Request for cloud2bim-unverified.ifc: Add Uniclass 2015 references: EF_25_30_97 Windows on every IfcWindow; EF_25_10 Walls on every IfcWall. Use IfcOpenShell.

First a look at what the model holds.

```python
import ifcopenshell

model = ifcopenshell.open("cloud2bim-unverified.ifc")
print(model.schema)
print("classifications:", [c.Name for c in model.by_type("IfcClassification")])
for ifc_class in ("IfcDoor", "IfcRoof", "IfcStair", "IfcWall", "IfcWindow"):
    print(ifc_class, len(model.by_type(ifc_class)))
```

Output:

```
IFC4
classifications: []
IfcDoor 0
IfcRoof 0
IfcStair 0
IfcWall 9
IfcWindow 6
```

```python
import ifcopenshell
import ifcopenshell.api.classification

model = ifcopenshell.open("cloud2bim-unverified.ifc")

system = ifcopenshell.api.classification.add_classification(model, classification="Uniclass 2015")

codes = {
    "IfcWindow": ("EF_25_30_97", "Windows"),
    "IfcWall": ("EF_25_10", "Walls"),
}
for ifc_class, (code, name) in codes.items():
    products = model.by_type(ifc_class)
    ifcopenshell.api.classification.add_reference(
        model, products=products, classification=system, identification=code, name=name
    )
    print(code, len(products))

model.write("cloud2bim-unverified_edited.ifc")
```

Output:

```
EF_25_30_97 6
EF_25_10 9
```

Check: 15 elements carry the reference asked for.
